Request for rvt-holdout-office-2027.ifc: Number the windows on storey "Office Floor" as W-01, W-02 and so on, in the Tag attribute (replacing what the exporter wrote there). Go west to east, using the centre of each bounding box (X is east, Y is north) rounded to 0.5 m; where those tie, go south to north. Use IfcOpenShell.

First a look at what the model holds.

```python
import ifcopenshell
import ifcopenshell.util.element
import ifcopenshell.util.placement

model = ifcopenshell.open("rvt-holdout-office-2027.ifc")
print(model.schema)
storey = next(s for s in model.by_type("IfcBuildingStorey") if s.Name == "Office Floor")
windows = [e for e in ifcopenshell.util.element.get_decomposition(storey) if e.is_a("IfcWindow")]
for e in sorted(windows, key=lambda e: e.id()):
    origin = ifcopenshell.util.placement.get_local_placement(e.ObjectPlacement)[:3, 3]
    print(e.id(), e.Tag, e.Name, origin.round(2) + 0.0, sep=" | ")
```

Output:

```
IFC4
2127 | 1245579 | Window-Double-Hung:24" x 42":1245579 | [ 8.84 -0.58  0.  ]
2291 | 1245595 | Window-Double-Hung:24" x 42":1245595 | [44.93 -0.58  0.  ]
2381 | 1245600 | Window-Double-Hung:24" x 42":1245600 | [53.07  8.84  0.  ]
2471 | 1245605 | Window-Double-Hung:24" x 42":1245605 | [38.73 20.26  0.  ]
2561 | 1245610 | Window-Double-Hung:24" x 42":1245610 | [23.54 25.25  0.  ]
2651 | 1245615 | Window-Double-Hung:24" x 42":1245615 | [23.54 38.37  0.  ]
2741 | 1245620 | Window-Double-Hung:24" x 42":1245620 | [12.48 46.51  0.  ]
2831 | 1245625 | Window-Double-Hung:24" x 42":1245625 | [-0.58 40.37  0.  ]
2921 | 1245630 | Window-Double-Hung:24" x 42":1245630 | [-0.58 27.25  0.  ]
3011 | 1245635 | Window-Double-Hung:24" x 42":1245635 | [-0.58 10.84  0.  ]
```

```python
import ifcopenshell
import ifcopenshell.geom
import ifcopenshell.util.element
import ifcopenshell.util.shape

model = ifcopenshell.open("rvt-holdout-office-2027.ifc")
settings = ifcopenshell.geom.settings()
settings.set("use-world-coords", True)


def centre(element):
    shape = ifcopenshell.geom.create_shape(settings, element)
    return ifcopenshell.util.shape.get_bbox_centroid(shape.geometry)


storey = next(s for s in model.by_type("IfcBuildingStorey") if s.Name == "Office Floor")
windows = [e for e in ifcopenshell.util.element.get_decomposition(storey) if e.is_a("IfcWindow")]

# Insertion points can sit at a corner or the storey origin, so sort by the geometry (in metres).
centres = {e: centre(e) for e in windows}
windows.sort(key=lambda e: (round(centres[e][0] / 0.5), centres[e][1]))

for i, e in enumerate(windows, start=1):
    number = f"W-{i:02d}"
    e.Tag = number
    print(e.id(), number)

model.write("rvt-holdout-office-2027_v2.ifc")
```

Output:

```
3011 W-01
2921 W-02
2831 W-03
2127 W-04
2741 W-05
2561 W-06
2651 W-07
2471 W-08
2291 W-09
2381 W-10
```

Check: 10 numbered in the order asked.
